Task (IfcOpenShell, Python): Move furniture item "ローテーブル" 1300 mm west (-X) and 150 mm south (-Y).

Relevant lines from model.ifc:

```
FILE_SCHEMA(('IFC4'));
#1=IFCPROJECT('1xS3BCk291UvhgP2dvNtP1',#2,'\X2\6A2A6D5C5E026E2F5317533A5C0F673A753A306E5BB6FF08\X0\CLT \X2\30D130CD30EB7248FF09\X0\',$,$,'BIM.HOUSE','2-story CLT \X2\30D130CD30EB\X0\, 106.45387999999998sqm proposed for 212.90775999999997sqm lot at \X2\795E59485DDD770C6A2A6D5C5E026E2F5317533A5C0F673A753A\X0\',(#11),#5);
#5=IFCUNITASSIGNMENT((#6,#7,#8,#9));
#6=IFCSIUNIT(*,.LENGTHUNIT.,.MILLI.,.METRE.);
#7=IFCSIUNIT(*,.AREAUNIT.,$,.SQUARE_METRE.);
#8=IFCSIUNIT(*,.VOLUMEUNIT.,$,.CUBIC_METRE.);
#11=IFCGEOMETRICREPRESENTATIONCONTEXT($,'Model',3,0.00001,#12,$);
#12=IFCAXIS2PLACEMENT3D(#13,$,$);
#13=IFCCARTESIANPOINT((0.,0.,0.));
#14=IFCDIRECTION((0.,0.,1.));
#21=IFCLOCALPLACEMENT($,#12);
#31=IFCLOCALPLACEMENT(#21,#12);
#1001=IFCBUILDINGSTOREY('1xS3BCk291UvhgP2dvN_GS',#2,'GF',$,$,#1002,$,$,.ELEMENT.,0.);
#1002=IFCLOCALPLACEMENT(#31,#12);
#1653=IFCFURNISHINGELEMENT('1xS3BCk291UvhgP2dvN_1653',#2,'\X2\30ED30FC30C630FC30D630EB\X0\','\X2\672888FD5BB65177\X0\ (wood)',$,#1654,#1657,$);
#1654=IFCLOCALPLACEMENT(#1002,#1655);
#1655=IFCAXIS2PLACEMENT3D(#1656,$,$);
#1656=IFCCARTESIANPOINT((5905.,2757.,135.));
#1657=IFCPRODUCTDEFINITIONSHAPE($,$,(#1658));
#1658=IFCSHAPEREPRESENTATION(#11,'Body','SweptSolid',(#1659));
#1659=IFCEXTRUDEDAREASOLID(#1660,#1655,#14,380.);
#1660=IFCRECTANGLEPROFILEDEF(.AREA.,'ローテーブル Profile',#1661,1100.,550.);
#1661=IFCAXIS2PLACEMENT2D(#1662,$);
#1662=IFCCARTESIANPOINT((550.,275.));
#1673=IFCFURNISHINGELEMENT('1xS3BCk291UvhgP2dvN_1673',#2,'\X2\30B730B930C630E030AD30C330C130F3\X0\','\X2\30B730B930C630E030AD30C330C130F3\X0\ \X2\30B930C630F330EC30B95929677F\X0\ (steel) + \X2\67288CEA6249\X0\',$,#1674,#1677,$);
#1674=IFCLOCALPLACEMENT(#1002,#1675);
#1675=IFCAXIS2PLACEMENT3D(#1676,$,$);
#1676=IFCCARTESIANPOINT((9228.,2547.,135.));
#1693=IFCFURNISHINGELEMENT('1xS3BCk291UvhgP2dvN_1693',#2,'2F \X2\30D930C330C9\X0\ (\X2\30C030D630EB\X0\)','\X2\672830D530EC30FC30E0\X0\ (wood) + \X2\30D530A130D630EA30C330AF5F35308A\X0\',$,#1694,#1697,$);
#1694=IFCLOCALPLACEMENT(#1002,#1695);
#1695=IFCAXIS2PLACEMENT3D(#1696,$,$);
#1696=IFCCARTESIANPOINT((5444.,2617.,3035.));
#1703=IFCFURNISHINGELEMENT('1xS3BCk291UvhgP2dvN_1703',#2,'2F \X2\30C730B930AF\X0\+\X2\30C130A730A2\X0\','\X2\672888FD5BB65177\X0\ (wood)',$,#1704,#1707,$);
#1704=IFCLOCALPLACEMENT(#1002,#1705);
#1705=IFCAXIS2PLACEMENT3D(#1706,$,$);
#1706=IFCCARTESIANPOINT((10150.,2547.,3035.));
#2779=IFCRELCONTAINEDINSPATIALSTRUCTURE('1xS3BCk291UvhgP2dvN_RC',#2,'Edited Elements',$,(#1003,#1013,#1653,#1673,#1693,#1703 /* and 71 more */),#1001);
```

```python
import ifcopenshell
import ifcopenshell.api.geometry
import ifcopenshell.util.placement
import ifcopenshell.util.unit

model = ifcopenshell.open("model.ifc")
unit_scale = ifcopenshell.util.unit.calculate_unit_scale(model)

item = model.by_id(1653)
matrix = ifcopenshell.util.placement.get_local_placement(item.ObjectPlacement)
matrix[0, 3] -= 1.3 / unit_scale
matrix[1, 3] -= 0.15 / unit_scale
ifcopenshell.api.geometry.edit_object_placement(model, product=item, matrix=matrix, is_si=False)

print(ifcopenshell.util.placement.get_local_placement(item.ObjectPlacement).round(3) + 0.0)

model.write("model_v2.ifc")
```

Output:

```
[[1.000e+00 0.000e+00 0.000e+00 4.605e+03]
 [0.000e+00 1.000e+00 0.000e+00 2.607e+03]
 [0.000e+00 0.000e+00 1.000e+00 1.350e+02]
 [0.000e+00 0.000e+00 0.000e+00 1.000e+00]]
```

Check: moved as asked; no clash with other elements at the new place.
